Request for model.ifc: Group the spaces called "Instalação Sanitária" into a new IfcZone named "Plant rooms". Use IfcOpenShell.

First a look at what the model holds.

```python
import ifcopenshell

model = ifcopenshell.open("model.ifc")
print(model.schema)
seen = {}
for space in model.by_type("IfcSpace"):
    seen[space.LongName] = seen.get(space.LongName, 0) + 1
for name, count in sorted(seen.items(), key=str):
    print(count, "x", name)
print("zones:", [z.Name for z in model.by_type("IfcZone")][:20])
```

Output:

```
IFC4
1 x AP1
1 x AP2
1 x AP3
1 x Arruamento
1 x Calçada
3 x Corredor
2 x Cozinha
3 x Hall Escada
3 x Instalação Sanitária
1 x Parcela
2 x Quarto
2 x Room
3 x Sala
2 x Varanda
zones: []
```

```python
import ifcopenshell
import ifcopenshell.api.group
import ifcopenshell.api.root

model = ifcopenshell.open("model.ifc")

names = {"Instalação Sanitária"}
spaces = [s for s in model.by_type("IfcSpace") if s.LongName in names]

zone = ifcopenshell.api.root.create_entity(model, ifc_class="IfcZone", name="Plant rooms")
ifcopenshell.api.group.assign_group(model, products=spaces, group=zone)
print(len(spaces), "spaces in", zone.Name)

model.write("model_edited.ifc")
```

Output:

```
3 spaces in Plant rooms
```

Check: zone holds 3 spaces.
